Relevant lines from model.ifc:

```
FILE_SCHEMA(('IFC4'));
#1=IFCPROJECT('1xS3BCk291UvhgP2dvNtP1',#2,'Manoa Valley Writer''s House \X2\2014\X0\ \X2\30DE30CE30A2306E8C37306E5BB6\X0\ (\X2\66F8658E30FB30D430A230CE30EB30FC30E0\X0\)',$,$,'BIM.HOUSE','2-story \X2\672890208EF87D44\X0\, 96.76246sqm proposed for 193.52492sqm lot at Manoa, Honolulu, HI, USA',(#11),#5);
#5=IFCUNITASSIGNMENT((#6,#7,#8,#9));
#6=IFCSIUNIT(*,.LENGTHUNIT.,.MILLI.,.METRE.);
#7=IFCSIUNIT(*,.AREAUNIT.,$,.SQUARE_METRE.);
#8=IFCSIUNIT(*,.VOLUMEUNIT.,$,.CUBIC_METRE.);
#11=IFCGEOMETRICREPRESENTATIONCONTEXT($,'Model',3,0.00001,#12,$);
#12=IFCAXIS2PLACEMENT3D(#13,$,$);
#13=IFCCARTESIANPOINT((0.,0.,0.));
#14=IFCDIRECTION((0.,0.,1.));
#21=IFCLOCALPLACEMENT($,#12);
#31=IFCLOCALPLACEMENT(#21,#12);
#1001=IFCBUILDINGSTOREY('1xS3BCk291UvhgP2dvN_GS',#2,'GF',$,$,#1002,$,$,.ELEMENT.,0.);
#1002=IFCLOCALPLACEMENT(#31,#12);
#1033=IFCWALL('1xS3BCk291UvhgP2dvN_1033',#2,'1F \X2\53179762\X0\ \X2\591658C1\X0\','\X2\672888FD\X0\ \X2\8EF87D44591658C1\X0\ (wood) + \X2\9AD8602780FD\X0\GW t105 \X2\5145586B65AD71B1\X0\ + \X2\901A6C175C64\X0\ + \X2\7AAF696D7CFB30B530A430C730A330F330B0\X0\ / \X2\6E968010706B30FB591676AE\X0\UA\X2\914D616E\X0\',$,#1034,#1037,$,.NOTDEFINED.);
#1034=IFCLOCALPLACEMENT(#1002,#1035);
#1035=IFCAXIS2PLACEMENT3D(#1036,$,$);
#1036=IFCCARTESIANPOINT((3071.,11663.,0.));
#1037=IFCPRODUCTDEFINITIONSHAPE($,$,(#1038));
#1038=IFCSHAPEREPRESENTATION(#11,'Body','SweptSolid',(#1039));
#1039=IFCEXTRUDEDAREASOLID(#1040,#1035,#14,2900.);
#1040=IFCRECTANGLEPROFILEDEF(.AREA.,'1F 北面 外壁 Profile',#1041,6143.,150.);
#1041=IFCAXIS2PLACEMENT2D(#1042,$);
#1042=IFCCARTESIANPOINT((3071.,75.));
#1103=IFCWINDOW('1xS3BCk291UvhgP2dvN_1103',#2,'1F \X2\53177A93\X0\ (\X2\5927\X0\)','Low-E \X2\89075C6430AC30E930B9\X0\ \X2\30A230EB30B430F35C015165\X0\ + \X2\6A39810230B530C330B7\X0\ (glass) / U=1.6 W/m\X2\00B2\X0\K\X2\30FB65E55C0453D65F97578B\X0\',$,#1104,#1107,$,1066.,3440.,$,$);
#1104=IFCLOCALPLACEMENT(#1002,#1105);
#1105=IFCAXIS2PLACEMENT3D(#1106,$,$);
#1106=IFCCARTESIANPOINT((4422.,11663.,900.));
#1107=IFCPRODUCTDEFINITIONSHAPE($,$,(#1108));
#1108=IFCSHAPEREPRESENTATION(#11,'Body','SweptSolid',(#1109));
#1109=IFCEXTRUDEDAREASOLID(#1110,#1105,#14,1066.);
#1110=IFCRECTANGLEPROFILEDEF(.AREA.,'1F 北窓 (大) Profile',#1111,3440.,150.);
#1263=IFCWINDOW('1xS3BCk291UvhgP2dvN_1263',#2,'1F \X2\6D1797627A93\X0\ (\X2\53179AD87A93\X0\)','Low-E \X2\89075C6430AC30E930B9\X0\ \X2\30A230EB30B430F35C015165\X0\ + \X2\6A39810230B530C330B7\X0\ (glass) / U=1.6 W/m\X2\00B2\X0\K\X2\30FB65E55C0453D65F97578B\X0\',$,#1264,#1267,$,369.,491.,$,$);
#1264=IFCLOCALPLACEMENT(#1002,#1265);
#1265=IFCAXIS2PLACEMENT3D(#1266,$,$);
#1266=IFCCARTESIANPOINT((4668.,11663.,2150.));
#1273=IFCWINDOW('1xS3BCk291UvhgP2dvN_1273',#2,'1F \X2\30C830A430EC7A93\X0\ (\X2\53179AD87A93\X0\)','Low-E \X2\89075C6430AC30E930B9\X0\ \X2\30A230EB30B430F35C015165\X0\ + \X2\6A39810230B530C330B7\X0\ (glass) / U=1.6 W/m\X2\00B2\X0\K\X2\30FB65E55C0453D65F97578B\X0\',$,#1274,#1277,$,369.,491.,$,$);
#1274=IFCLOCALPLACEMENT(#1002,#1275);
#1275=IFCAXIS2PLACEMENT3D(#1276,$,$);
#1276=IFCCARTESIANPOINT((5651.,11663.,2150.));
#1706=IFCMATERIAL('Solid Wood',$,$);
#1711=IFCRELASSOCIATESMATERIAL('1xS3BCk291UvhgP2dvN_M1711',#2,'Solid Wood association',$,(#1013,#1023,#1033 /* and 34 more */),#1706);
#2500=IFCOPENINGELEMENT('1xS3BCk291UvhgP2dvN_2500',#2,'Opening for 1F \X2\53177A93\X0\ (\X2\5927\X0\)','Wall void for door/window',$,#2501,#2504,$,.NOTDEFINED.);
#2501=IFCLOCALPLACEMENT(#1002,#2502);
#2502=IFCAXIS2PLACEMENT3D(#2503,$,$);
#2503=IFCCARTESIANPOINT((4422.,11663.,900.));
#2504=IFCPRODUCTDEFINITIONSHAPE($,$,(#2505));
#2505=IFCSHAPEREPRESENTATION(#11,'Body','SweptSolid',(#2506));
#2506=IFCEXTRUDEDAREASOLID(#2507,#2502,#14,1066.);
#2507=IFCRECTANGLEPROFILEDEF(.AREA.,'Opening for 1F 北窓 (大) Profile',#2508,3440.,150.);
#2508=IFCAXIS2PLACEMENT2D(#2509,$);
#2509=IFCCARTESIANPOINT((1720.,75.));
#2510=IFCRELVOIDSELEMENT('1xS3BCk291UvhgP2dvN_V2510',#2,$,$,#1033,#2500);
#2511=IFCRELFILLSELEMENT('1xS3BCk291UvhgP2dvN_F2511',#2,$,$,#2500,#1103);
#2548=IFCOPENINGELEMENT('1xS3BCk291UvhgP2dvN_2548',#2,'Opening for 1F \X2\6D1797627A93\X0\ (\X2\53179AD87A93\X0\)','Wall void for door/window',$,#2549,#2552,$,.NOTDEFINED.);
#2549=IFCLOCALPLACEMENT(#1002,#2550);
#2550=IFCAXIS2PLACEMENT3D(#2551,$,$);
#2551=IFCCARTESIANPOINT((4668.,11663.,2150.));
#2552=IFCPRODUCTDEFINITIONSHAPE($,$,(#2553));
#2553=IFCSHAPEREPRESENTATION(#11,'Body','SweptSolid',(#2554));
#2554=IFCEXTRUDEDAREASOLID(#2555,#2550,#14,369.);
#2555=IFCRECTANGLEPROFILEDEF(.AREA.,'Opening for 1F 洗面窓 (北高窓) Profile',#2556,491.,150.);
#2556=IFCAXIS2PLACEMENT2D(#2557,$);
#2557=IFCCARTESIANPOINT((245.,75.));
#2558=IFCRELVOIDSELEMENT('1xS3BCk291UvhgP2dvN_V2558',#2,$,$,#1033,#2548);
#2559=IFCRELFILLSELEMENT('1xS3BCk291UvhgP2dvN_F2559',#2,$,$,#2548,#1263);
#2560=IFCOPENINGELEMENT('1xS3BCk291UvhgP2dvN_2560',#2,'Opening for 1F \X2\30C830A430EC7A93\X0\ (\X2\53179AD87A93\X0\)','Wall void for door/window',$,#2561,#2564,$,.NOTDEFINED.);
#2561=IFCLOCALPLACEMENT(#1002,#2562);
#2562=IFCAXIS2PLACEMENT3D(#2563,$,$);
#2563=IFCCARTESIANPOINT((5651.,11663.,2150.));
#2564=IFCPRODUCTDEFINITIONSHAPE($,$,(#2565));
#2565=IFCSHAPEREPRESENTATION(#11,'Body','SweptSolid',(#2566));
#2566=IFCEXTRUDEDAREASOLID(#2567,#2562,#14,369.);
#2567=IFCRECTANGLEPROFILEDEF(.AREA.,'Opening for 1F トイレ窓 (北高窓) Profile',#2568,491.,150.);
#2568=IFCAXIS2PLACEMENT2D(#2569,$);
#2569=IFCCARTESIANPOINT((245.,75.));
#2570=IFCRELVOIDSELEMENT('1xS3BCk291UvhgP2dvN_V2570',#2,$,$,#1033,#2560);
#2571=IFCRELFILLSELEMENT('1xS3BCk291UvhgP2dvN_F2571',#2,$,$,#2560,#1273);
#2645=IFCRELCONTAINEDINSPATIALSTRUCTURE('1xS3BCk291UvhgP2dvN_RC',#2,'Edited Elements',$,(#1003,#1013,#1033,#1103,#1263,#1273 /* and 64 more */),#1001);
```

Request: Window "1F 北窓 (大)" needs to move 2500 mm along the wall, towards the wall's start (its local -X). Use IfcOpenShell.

```python
import ifcopenshell
import ifcopenshell.api.geometry
import ifcopenshell.util.placement

model = ifcopenshell.open("model.ifc")

window = model.by_guid("1xS3BCk291UvhgP2dvN_1103")
opening = window.FillsVoids[0].RelatingOpeningElement
wall = opening.VoidsElements[0].RelatingBuildingElement

wall_matrix = ifcopenshell.util.placement.get_local_placement(wall.ObjectPlacement)
shift = wall_matrix[:3, 0] * -2500.0
before = ifcopenshell.util.placement.get_local_placement(window.ObjectPlacement)[:3, 3].copy()

# The window is not placed relative to its opening, so move both.
for product in (opening, window):
    matrix = ifcopenshell.util.placement.get_local_placement(product.ObjectPlacement)
    matrix[:3, 3] += shift
    ifcopenshell.api.geometry.edit_object_placement(model, product=product, matrix=matrix, is_si=False)

after = ifcopenshell.util.placement.get_local_placement(window.ObjectPlacement)[:3, 3]
print("window moved by", (after - before).round(3) + 0.0)

model.write("model_updated.ifc")
```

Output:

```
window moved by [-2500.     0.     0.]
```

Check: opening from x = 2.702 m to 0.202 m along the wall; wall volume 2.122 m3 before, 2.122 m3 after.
